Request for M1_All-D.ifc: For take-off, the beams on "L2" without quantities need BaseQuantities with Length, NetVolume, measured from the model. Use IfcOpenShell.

First a look at what the model holds.

```python
import ifcopenshell
import ifcopenshell.util.element
import ifcopenshell.util.unit

model = ifcopenshell.open("M1_All-D.ifc")
print(model.schema)
for unit_type in ("LENGTHUNIT", "AREAUNIT", "VOLUMEUNIT"):
    print(unit_type, ifcopenshell.util.unit.calculate_unit_scale(model, unit_type))
storey = next(s for s in model.by_type("IfcBuildingStorey") if s.Name == "L2")
beams = [e for e in ifcopenshell.util.element.get_decomposition(storey) if e.is_a("IfcBeam")]
for e in sorted(beams, key=lambda e: e.id()):
    print(e.id(), e.is_a(), e.Name, list(ifcopenshell.util.element.get_psets(e, qtos_only=True)), sep=" | ")
```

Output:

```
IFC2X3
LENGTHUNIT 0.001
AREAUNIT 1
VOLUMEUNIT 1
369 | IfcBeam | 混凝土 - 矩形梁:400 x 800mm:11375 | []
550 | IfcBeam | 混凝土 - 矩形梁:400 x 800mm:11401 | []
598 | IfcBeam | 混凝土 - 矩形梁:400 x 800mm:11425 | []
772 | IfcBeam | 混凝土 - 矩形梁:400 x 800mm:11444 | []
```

```python
import ifcopenshell
import ifcopenshell.api.pset
import ifcopenshell.geom
import ifcopenshell.util.element
import ifcopenshell.util.shape
import ifcopenshell.util.unit

model = ifcopenshell.open("M1_All-D.ifc")
unit_scale = ifcopenshell.util.unit.calculate_unit_scale(model)
volume_scale = ifcopenshell.util.unit.calculate_unit_scale(model, "VOLUMEUNIT")
settings = ifcopenshell.geom.settings()

storey = next(s for s in model.by_type("IfcBuildingStorey") if s.Name == "L2")
beams = [e for e in ifcopenshell.util.element.get_decomposition(storey) if e.is_a("IfcBeam")]

for e in sorted(beams, key=lambda e: e.id()):
    if ifcopenshell.util.element.get_psets(e, qtos_only=True, should_inherit=False):
        continue
    # Geometry comes back in metres, in the element's own axes.
    shape = ifcopenshell.geom.create_shape(settings, e)
    values = {
        "Length": ifcopenshell.util.shape.get_max_xyz(shape.geometry) / unit_scale,
        "NetVolume": ifcopenshell.util.shape.get_volume(shape.geometry) / volume_scale,
    }
    qto = ifcopenshell.api.pset.add_qto(model, product=e, name="BaseQuantities")
    ifcopenshell.api.pset.edit_qto(model, qto=qto, properties=values)
    print(e.id(), {k: round(v, 3) for k, v in values.items()})

model.write("M1_All-D_edited.ifc")
```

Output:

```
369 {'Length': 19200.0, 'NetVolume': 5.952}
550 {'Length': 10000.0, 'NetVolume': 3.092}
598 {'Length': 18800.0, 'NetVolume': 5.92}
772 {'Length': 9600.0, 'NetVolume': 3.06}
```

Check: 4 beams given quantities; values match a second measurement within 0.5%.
